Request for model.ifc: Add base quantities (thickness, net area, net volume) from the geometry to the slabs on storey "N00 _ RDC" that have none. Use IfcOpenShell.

First a look at what the model holds.

```python
import ifcopenshell
import ifcopenshell.util.element
import ifcopenshell.util.unit

model = ifcopenshell.open("model.ifc")
print(model.schema)
for unit_type in ("LENGTHUNIT", "AREAUNIT", "VOLUMEUNIT"):
    print(unit_type, ifcopenshell.util.unit.calculate_unit_scale(model, unit_type))
storey = next(s for s in model.by_type("IfcBuildingStorey") if s.Name == "N00 _ RDC")
slabs = [e for e in ifcopenshell.util.element.get_decomposition(storey) if e.is_a("IfcSlab")]
for e in sorted(slabs, key=lambda e: e.id()):
    print(e.id(), e.is_a(), e.Name, list(ifcopenshell.util.element.get_psets(e, qtos_only=True)), sep=" | ")
```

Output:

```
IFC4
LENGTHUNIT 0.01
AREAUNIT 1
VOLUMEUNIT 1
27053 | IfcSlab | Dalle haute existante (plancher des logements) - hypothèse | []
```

```python
import ifcopenshell
import ifcopenshell.api.pset
import ifcopenshell.geom
import ifcopenshell.util.element
import ifcopenshell.util.shape
import ifcopenshell.util.unit

model = ifcopenshell.open("model.ifc")
unit_scale = ifcopenshell.util.unit.calculate_unit_scale(model)
area_scale = ifcopenshell.util.unit.calculate_unit_scale(model, "AREAUNIT")
volume_scale = ifcopenshell.util.unit.calculate_unit_scale(model, "VOLUMEUNIT")
settings = ifcopenshell.geom.settings()

storey = next(s for s in model.by_type("IfcBuildingStorey") if s.Name == "N00 _ RDC")
slabs = [e for e in ifcopenshell.util.element.get_decomposition(storey) if e.is_a("IfcSlab")]

for e in sorted(slabs, key=lambda e: e.id()):
    if ifcopenshell.util.element.get_psets(e, qtos_only=True, should_inherit=False):
        continue
    # Geometry comes back in metres, in the element's own axes.
    shape = ifcopenshell.geom.create_shape(settings, e)
    values = {
        "Width": ifcopenshell.util.shape.get_z(shape.geometry) / unit_scale,
        "NetArea": ifcopenshell.util.shape.get_footprint_area(shape.geometry) / area_scale,
        "NetVolume": ifcopenshell.util.shape.get_volume(shape.geometry) / volume_scale,
    }
    qto = ifcopenshell.api.pset.add_qto(model, product=e, name="Qto_SlabBaseQuantities")
    ifcopenshell.api.pset.edit_qto(model, qto=qto, properties=values)
    print(e.id(), {k: round(v, 3) for k, v in values.items()})

model.write("model_updated.ifc")
```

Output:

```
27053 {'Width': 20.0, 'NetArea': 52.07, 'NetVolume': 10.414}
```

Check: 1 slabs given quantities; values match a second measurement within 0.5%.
